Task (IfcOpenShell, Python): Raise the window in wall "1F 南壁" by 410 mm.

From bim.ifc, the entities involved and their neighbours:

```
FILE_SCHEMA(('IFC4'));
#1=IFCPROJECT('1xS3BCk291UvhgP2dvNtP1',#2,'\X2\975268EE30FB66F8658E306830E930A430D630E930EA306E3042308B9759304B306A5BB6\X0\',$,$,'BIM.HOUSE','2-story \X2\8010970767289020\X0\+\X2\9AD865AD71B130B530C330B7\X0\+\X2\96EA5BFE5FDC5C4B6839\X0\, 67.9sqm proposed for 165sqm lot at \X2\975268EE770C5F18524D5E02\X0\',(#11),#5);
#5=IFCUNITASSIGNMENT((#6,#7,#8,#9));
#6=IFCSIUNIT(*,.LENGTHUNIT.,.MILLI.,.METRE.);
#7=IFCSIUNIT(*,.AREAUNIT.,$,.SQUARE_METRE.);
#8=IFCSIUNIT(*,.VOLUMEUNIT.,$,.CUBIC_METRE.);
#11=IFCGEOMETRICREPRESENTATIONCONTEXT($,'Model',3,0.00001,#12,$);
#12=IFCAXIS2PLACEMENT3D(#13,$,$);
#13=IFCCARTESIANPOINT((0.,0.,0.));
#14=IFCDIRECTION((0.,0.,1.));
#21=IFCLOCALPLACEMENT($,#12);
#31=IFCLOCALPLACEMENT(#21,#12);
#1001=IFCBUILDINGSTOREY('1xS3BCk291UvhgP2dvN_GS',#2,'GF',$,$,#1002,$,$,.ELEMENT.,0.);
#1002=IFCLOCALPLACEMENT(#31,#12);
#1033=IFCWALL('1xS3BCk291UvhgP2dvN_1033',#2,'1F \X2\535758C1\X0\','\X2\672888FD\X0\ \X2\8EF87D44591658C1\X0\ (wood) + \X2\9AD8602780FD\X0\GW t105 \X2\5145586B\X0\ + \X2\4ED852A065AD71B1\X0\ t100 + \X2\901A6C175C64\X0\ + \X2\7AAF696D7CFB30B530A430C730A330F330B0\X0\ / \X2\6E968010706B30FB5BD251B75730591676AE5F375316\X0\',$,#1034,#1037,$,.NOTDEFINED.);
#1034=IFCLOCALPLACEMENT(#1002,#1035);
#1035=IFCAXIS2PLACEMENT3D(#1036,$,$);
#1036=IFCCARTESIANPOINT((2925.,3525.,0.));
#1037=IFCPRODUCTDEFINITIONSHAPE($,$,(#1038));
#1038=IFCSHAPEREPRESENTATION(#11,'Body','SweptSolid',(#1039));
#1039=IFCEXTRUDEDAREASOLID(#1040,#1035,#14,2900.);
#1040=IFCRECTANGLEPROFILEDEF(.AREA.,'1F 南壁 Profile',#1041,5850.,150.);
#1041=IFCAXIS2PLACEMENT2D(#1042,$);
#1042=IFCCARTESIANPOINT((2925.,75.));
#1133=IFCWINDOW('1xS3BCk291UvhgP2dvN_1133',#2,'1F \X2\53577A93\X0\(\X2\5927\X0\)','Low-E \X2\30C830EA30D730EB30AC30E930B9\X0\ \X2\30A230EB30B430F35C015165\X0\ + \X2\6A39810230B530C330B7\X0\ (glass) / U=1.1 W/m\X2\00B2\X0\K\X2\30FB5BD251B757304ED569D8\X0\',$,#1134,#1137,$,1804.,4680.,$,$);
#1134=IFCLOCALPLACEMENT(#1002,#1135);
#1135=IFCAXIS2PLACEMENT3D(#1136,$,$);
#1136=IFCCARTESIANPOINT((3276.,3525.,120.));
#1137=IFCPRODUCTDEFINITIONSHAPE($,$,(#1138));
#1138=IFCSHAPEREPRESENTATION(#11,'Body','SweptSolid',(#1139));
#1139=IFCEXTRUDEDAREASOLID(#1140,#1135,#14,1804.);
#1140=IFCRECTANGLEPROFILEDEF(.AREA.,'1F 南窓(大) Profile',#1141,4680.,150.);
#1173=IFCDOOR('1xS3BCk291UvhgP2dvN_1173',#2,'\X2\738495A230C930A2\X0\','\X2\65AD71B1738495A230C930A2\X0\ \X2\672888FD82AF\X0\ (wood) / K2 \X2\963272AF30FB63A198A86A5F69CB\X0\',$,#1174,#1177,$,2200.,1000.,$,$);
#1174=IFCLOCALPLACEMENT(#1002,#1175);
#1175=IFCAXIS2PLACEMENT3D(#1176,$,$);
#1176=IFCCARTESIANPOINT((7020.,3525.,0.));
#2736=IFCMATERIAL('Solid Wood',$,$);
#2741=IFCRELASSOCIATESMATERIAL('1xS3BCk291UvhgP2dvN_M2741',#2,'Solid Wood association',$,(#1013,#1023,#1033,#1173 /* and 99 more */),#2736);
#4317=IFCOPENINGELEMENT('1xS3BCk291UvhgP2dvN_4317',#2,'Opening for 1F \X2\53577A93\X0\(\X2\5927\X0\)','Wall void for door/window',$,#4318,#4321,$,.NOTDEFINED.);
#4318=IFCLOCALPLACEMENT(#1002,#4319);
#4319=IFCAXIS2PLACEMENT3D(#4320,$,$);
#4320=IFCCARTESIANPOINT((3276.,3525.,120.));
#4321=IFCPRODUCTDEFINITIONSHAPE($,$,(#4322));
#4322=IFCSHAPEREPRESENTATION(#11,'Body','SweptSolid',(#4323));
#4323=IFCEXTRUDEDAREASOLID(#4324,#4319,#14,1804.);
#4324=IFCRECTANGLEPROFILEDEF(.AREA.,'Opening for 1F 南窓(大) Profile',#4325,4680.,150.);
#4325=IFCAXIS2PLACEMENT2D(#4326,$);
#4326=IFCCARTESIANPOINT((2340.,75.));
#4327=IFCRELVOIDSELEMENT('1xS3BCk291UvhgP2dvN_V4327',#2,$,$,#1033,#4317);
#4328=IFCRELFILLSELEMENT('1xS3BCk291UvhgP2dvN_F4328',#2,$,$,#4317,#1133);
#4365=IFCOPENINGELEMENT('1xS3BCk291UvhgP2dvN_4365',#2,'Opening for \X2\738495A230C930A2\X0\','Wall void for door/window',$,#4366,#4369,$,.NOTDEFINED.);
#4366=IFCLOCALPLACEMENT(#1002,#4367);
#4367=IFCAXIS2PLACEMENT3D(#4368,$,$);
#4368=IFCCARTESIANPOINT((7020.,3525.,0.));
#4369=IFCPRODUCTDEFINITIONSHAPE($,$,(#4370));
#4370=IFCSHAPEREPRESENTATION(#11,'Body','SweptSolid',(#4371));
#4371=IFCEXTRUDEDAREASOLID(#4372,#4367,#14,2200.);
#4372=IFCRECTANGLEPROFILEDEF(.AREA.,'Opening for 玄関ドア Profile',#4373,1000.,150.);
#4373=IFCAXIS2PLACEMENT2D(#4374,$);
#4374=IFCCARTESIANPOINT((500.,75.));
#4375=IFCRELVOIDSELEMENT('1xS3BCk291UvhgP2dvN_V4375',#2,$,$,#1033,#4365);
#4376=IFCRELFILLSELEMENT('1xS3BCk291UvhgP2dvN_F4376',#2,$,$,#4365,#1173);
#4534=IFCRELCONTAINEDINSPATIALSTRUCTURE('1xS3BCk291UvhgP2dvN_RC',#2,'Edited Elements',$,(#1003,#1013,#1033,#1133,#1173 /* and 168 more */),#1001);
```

```python
import numpy as np
import ifcopenshell
import ifcopenshell.api.geometry
import ifcopenshell.util.placement
import ifcopenshell.util.unit

model = ifcopenshell.open("bim.ifc")
unit_scale = ifcopenshell.util.unit.calculate_unit_scale(model)

window = model.by_id(1133)
opening = window.FillsVoids[0].RelatingOpeningElement
dz = 410.0

shift = np.array([0.0, 0.0, dz])
# The window is not placed relative to its opening, so move both.
for product in (opening, window):
    matrix = ifcopenshell.util.placement.get_local_placement(product.ObjectPlacement)
    matrix[:3, 3] += shift
    ifcopenshell.api.geometry.edit_object_placement(model, product=product, matrix=matrix, is_si=False)

print(f"moved by {dz * unit_scale:+.3f} m")

model.write("bim_v2.ifc")
```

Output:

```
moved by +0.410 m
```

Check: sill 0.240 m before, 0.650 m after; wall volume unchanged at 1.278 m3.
